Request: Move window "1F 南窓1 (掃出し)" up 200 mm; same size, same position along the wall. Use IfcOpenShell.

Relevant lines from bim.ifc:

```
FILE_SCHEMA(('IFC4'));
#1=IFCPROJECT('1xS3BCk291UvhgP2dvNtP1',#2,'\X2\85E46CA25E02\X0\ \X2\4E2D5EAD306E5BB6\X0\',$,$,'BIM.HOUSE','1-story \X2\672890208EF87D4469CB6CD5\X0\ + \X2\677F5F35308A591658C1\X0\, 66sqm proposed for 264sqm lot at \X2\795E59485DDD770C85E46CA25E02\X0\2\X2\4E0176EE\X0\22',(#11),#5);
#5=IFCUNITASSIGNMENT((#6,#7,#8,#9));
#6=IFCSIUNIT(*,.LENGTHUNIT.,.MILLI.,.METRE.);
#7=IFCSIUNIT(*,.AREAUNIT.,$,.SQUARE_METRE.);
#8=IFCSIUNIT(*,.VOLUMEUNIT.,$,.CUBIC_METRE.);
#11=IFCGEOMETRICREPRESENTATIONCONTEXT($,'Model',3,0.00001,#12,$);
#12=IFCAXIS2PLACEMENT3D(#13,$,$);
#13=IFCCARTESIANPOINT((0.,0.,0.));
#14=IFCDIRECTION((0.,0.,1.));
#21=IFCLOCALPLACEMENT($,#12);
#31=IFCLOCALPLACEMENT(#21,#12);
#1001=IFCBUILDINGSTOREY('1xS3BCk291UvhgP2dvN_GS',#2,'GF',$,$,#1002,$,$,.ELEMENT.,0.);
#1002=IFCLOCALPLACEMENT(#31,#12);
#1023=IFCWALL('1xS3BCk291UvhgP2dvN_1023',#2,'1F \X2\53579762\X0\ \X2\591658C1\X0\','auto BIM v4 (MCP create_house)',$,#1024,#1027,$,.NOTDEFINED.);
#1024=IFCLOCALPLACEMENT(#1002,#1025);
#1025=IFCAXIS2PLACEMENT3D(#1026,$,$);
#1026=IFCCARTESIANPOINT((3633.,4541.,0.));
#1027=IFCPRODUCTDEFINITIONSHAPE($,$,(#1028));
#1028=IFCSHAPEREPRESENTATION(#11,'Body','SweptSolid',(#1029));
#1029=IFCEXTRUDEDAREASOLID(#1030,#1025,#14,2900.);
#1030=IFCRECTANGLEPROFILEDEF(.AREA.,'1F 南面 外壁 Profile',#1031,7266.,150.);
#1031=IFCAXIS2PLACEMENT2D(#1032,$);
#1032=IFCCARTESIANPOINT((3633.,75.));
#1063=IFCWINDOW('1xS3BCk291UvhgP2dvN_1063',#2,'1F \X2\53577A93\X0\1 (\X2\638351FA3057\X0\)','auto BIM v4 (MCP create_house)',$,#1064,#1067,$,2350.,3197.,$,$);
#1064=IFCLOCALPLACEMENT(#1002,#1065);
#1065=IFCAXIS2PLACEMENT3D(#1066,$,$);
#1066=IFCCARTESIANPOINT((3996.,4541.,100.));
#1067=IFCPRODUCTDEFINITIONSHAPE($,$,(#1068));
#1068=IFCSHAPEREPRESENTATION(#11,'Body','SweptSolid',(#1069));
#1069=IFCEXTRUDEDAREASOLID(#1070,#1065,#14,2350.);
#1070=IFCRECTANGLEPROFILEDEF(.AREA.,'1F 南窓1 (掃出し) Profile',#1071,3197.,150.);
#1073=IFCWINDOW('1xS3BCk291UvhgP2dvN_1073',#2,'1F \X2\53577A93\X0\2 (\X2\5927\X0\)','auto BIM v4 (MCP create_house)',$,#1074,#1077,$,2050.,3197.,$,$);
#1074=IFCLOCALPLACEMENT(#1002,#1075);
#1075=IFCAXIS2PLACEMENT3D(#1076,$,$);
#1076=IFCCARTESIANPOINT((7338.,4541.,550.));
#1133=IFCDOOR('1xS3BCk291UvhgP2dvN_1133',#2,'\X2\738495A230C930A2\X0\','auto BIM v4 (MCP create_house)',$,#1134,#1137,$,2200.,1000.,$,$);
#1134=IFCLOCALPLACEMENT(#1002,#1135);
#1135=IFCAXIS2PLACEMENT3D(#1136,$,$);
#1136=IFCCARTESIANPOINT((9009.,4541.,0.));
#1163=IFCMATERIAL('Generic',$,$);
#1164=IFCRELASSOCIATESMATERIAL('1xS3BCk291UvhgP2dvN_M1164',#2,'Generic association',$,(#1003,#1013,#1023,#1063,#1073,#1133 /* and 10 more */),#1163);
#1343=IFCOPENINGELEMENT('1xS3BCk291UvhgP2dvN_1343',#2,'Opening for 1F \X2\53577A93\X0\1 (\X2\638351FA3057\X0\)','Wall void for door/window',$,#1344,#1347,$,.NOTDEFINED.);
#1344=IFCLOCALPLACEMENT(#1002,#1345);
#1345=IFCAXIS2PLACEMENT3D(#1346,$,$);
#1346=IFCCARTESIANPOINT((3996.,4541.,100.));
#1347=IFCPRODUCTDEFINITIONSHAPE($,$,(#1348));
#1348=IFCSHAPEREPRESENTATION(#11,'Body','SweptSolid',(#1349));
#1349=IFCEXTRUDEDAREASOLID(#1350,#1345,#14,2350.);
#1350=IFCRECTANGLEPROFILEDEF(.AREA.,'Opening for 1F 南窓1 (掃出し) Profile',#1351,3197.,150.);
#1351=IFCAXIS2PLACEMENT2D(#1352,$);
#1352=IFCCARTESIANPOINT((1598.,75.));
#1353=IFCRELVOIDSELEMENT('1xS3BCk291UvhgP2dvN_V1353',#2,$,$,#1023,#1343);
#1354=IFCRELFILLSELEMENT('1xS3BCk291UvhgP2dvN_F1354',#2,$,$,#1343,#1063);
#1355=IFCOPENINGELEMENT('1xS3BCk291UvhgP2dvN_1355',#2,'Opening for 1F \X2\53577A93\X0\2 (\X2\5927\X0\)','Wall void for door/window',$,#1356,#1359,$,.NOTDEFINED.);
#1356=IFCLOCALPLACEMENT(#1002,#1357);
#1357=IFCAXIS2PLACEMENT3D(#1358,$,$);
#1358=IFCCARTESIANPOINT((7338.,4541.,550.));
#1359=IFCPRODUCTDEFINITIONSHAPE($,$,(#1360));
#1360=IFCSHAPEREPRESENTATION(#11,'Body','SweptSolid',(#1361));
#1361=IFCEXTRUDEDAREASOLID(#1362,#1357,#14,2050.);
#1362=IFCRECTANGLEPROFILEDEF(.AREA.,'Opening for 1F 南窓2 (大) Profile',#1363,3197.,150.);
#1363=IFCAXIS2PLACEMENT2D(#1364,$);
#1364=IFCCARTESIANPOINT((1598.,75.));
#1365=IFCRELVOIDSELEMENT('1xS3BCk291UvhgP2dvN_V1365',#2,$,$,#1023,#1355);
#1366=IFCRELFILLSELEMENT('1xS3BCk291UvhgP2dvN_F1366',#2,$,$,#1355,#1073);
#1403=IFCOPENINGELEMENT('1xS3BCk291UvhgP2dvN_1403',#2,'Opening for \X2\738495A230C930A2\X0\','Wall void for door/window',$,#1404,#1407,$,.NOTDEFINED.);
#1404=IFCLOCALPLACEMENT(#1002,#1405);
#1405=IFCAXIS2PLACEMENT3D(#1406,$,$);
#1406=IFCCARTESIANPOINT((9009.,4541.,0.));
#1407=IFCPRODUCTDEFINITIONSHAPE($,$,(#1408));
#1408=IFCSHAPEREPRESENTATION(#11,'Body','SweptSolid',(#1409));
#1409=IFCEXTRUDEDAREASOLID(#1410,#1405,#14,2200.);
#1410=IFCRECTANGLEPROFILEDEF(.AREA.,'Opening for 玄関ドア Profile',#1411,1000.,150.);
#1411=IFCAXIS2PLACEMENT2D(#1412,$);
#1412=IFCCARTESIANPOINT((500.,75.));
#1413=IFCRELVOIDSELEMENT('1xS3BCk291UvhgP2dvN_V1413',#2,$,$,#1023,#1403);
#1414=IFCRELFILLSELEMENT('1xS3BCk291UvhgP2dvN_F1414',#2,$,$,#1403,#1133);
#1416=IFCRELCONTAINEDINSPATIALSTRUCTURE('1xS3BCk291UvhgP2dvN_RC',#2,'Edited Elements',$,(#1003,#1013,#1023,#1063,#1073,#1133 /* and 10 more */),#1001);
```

```python
import numpy as np
import ifcopenshell
import ifcopenshell.api.geometry
import ifcopenshell.util.placement
import ifcopenshell.util.unit

model = ifcopenshell.open("bim.ifc")
unit_scale = ifcopenshell.util.unit.calculate_unit_scale(model)

window = model.by_id(1063)
opening = window.FillsVoids[0].RelatingOpeningElement
dz = 0.2 / unit_scale

shift = np.array([0.0, 0.0, dz])
# The window is not placed relative to its opening, so move both.
for product in (opening, window):
    matrix = ifcopenshell.util.placement.get_local_placement(product.ObjectPlacement)
    matrix[:3, 3] += shift
    ifcopenshell.api.geometry.edit_object_placement(model, product=product, matrix=matrix, is_si=False)

print(f"moved by {dz * unit_scale:+.3f} m")

model.write("bim_updated.ifc")
```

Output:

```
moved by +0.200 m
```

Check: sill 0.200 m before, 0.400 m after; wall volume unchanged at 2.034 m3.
